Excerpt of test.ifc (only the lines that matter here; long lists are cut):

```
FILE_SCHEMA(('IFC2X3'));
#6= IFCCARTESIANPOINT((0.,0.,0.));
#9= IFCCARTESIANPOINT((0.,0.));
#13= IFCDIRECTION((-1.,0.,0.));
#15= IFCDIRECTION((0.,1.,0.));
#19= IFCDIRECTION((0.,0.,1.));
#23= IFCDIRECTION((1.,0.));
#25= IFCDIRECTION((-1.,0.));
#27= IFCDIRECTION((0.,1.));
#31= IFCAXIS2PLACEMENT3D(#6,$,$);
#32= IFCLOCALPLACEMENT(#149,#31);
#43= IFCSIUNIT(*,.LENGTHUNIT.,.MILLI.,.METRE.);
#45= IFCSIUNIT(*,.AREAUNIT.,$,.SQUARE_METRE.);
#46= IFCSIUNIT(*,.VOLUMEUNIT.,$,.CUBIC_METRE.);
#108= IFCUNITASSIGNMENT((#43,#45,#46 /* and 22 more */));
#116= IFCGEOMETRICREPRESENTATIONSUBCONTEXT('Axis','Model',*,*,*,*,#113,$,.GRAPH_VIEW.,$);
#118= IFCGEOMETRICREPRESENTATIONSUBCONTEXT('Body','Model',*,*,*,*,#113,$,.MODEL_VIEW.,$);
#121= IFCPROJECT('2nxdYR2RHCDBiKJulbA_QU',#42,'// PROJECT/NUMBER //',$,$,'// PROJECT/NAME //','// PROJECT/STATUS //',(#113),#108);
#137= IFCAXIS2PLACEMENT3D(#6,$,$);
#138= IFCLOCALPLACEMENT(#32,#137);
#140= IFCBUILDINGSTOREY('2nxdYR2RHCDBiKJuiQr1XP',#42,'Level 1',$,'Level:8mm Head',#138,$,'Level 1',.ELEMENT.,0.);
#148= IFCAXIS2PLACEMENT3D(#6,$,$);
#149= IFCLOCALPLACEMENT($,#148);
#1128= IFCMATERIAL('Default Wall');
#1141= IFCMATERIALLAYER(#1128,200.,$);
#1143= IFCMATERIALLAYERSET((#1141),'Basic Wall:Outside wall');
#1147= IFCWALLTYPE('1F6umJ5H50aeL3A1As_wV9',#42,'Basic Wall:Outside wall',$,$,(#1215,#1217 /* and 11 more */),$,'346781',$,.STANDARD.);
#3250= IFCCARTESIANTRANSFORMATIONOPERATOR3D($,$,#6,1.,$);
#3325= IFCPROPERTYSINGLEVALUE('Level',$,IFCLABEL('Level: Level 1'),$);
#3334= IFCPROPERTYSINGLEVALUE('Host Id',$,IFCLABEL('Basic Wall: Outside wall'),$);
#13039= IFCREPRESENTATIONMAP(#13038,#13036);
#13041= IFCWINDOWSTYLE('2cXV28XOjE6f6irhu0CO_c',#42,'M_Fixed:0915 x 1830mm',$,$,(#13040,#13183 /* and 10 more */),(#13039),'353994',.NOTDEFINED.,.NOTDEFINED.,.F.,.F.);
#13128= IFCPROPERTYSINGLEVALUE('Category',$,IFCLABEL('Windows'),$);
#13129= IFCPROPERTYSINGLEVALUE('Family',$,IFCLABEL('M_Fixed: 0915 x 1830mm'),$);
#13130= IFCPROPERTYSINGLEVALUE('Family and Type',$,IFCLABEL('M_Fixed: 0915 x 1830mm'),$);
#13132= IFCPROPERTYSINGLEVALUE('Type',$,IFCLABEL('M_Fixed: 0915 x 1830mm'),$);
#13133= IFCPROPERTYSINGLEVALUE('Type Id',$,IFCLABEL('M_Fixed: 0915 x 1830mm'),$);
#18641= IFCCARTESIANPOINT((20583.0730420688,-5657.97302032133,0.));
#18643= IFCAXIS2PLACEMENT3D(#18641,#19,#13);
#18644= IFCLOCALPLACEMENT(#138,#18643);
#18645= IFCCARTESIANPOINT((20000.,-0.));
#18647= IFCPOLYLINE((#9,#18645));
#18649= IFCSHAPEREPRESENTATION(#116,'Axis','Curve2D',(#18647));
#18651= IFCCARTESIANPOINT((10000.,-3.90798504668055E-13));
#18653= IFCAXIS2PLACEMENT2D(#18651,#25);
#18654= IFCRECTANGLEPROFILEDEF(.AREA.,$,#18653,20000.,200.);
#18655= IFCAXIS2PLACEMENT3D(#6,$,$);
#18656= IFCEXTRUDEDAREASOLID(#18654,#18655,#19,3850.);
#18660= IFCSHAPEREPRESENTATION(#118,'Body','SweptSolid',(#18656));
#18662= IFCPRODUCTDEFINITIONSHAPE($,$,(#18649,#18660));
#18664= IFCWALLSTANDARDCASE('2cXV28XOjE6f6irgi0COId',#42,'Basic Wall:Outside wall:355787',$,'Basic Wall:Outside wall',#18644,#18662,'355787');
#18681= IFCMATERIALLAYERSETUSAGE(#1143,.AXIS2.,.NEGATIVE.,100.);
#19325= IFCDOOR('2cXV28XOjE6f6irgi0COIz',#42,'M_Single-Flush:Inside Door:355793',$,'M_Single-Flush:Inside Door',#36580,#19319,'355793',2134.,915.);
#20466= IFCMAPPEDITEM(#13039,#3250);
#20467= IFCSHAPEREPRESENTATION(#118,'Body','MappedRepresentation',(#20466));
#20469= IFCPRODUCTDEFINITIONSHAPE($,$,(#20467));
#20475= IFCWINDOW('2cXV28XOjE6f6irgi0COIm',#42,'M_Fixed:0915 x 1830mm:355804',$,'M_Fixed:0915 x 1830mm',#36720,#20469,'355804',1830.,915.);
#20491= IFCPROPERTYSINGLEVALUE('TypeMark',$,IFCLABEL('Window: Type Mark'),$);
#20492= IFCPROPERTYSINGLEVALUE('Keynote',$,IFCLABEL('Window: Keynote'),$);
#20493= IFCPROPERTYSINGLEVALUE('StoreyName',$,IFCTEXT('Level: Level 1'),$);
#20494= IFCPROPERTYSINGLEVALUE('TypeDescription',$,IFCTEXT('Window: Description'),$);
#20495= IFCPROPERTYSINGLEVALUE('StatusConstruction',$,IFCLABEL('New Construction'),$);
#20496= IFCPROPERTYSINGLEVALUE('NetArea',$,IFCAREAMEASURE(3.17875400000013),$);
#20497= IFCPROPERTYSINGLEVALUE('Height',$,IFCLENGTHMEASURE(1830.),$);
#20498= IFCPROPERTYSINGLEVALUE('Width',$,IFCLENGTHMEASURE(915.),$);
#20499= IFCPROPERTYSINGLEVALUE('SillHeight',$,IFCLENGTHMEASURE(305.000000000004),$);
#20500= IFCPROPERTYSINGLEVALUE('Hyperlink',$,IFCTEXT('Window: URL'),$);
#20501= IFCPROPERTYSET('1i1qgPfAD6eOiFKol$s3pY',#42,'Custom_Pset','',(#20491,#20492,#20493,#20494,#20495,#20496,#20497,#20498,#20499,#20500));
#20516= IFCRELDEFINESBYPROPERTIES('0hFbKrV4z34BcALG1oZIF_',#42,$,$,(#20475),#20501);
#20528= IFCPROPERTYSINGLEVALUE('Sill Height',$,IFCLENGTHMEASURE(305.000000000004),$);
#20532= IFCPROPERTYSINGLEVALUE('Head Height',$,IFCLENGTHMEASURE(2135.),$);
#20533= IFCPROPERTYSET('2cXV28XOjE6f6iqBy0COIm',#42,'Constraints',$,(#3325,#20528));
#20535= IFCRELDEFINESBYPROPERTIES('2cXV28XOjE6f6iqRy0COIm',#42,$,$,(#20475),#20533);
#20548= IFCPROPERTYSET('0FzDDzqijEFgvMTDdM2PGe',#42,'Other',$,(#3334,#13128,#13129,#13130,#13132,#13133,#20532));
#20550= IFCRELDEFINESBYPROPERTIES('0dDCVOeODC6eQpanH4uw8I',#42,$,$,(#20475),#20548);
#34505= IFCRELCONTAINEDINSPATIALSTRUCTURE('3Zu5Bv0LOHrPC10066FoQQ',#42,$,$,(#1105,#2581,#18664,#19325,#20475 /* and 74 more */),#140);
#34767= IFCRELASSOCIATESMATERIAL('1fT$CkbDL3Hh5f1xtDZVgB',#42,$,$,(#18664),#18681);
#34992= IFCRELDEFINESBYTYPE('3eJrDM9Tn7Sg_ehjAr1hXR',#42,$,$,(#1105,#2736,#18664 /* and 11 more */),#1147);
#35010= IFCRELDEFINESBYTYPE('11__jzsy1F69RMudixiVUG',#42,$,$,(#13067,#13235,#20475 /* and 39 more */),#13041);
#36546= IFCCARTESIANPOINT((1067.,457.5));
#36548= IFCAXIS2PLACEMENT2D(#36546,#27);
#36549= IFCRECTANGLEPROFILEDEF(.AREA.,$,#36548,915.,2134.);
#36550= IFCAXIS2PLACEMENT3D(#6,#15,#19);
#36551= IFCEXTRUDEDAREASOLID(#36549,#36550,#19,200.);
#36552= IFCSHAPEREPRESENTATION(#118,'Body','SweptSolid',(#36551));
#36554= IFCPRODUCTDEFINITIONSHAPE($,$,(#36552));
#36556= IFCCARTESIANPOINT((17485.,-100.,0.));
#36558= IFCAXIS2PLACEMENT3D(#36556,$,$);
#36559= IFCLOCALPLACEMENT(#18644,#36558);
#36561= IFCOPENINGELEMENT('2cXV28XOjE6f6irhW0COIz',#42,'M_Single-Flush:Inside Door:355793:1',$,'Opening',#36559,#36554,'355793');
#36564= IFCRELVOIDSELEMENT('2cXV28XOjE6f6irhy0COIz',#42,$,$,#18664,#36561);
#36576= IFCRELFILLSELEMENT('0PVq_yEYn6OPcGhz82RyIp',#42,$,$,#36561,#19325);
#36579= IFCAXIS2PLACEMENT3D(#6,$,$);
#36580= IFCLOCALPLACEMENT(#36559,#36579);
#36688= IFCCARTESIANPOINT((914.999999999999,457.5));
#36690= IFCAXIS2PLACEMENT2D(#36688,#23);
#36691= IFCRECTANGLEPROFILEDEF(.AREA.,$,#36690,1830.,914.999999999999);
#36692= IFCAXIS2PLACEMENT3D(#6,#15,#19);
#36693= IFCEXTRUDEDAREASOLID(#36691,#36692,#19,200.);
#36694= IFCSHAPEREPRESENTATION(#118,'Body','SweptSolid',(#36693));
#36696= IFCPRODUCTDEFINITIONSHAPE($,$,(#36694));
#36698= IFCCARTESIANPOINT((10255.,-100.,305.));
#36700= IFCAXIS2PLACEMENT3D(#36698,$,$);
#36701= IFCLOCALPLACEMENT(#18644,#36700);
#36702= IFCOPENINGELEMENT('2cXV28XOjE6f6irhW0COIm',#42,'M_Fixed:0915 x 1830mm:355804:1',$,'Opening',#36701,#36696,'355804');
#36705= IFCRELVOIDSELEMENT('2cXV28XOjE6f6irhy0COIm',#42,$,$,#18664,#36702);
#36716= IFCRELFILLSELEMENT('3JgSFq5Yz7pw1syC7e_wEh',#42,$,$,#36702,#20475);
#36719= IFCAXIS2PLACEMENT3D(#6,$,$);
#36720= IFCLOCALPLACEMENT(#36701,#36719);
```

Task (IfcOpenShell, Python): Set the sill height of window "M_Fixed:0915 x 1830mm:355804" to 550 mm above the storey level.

```python
import numpy as np
import ifcopenshell
import ifcopenshell.api.geometry
import ifcopenshell.api.pset
import ifcopenshell.geom
import ifcopenshell.util.element
import ifcopenshell.util.placement
import ifcopenshell.util.shape
import ifcopenshell.util.unit

model = ifcopenshell.open("test.ifc")
unit_scale = ifcopenshell.util.unit.calculate_unit_scale(model)

window = model.by_guid("2cXV28XOjE6f6irgi0COIm")
opening = window.FillsVoids[0].RelatingOpeningElement
storey = ifcopenshell.util.element.get_container(window, ifc_class="IfcBuildingStorey")
level = ifcopenshell.util.placement.get_local_placement(storey.ObjectPlacement)[2, 3]

# The opening's origin need not be at the sill, so measure its lowest point.
shape = ifcopenshell.geom.create_shape(ifcopenshell.geom.settings(), opening)
bottom = ifcopenshell.util.shape.get_shape_bottom_elevation(shape, shape.geometry) / unit_scale
dz = level + 0.55 / unit_scale - bottom

shift = np.array([0.0, 0.0, dz])
# The window is placed relative to its opening, so it follows when the opening moves.
matrix = ifcopenshell.util.placement.get_local_placement(opening.ObjectPlacement)
matrix[:3, 3] += shift
ifcopenshell.api.geometry.edit_object_placement(
    model, product=opening, matrix=matrix, is_si=False, should_transform_children=True
)

# Keep the stored heights in step.
pset = model.by_id(ifcopenshell.util.element.get_pset(window, "Custom_Pset", should_inherit=False)["id"])
ifcopenshell.api.pset.edit_pset(model, pset=pset, properties={
    "SillHeight": model.create_entity("IfcLengthMeasure", ifcopenshell.util.element.get_pset(window, "Constraints", "Sill Height") + dz),
})
pset = model.by_id(ifcopenshell.util.element.get_pset(window, "Constraints", should_inherit=False)["id"])
ifcopenshell.api.pset.edit_pset(model, pset=pset, properties={
    "Sill Height": model.create_entity("IfcLengthMeasure", ifcopenshell.util.element.get_pset(window, "Constraints", "Sill Height") + dz),
})
pset = model.by_id(ifcopenshell.util.element.get_pset(window, "Other", should_inherit=False)["id"])
ifcopenshell.api.pset.edit_pset(model, pset=pset, properties={
    "Head Height": model.create_entity("IfcLengthMeasure", ifcopenshell.util.element.get_pset(window, "Other", "Head Height") + dz),
})

print(f"moved by {dz * unit_scale:+.3f} m")

model.write("test_updated.ifc")
```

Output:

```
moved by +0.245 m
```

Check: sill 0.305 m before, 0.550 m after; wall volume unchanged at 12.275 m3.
